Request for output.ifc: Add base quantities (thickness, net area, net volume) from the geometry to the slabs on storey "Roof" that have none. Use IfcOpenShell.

First a look at what the model holds.

```python
import ifcopenshell
import ifcopenshell.util.element
import ifcopenshell.util.unit

model = ifcopenshell.open("output.ifc")
print(model.schema)
for unit_type in ("LENGTHUNIT", "AREAUNIT", "VOLUMEUNIT"):
    print(unit_type, ifcopenshell.util.unit.calculate_unit_scale(model, unit_type))
storey = next(s for s in model.by_type("IfcBuildingStorey") if s.Name == "Roof")
slabs = [e for e in ifcopenshell.util.element.get_decomposition(storey) if e.is_a("IfcSlab")]
for e in sorted(slabs, key=lambda e: e.id()):
    print(e.id(), e.is_a(), e.Name, list(ifcopenshell.util.element.get_psets(e, qtos_only=True)), sep=" | ")
```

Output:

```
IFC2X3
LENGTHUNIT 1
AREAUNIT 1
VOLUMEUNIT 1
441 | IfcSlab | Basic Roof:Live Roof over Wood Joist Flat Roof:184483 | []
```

```python
import ifcopenshell
import ifcopenshell.api.pset
import ifcopenshell.geom
import ifcopenshell.util.element
import ifcopenshell.util.shape
import ifcopenshell.util.unit

model = ifcopenshell.open("output.ifc")
unit_scale = ifcopenshell.util.unit.calculate_unit_scale(model)
area_scale = ifcopenshell.util.unit.calculate_unit_scale(model, "AREAUNIT")
volume_scale = ifcopenshell.util.unit.calculate_unit_scale(model, "VOLUMEUNIT")
settings = ifcopenshell.geom.settings()

storey = next(s for s in model.by_type("IfcBuildingStorey") if s.Name == "Roof")
slabs = [e for e in ifcopenshell.util.element.get_decomposition(storey) if e.is_a("IfcSlab")]

for e in sorted(slabs, key=lambda e: e.id()):
    if ifcopenshell.util.element.get_psets(e, qtos_only=True, should_inherit=False):
        continue
    # Geometry comes back in metres, in the element's own axes.
    shape = ifcopenshell.geom.create_shape(settings, e)
    values = {
        "Width": ifcopenshell.util.shape.get_z(shape.geometry) / unit_scale,
        "NetArea": ifcopenshell.util.shape.get_footprint_area(shape.geometry) / area_scale,
        "NetVolume": ifcopenshell.util.shape.get_volume(shape.geometry) / volume_scale,
    }
    qto = ifcopenshell.api.pset.add_qto(model, product=e, name="BaseQuantities")
    ifcopenshell.api.pset.edit_qto(model, qto=qto, properties=values)
    print(e.id(), {k: round(v, 3) for k, v in values.items()})

model.write("output_updated.ifc")
```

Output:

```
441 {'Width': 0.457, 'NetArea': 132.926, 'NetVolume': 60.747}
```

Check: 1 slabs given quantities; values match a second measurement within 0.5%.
